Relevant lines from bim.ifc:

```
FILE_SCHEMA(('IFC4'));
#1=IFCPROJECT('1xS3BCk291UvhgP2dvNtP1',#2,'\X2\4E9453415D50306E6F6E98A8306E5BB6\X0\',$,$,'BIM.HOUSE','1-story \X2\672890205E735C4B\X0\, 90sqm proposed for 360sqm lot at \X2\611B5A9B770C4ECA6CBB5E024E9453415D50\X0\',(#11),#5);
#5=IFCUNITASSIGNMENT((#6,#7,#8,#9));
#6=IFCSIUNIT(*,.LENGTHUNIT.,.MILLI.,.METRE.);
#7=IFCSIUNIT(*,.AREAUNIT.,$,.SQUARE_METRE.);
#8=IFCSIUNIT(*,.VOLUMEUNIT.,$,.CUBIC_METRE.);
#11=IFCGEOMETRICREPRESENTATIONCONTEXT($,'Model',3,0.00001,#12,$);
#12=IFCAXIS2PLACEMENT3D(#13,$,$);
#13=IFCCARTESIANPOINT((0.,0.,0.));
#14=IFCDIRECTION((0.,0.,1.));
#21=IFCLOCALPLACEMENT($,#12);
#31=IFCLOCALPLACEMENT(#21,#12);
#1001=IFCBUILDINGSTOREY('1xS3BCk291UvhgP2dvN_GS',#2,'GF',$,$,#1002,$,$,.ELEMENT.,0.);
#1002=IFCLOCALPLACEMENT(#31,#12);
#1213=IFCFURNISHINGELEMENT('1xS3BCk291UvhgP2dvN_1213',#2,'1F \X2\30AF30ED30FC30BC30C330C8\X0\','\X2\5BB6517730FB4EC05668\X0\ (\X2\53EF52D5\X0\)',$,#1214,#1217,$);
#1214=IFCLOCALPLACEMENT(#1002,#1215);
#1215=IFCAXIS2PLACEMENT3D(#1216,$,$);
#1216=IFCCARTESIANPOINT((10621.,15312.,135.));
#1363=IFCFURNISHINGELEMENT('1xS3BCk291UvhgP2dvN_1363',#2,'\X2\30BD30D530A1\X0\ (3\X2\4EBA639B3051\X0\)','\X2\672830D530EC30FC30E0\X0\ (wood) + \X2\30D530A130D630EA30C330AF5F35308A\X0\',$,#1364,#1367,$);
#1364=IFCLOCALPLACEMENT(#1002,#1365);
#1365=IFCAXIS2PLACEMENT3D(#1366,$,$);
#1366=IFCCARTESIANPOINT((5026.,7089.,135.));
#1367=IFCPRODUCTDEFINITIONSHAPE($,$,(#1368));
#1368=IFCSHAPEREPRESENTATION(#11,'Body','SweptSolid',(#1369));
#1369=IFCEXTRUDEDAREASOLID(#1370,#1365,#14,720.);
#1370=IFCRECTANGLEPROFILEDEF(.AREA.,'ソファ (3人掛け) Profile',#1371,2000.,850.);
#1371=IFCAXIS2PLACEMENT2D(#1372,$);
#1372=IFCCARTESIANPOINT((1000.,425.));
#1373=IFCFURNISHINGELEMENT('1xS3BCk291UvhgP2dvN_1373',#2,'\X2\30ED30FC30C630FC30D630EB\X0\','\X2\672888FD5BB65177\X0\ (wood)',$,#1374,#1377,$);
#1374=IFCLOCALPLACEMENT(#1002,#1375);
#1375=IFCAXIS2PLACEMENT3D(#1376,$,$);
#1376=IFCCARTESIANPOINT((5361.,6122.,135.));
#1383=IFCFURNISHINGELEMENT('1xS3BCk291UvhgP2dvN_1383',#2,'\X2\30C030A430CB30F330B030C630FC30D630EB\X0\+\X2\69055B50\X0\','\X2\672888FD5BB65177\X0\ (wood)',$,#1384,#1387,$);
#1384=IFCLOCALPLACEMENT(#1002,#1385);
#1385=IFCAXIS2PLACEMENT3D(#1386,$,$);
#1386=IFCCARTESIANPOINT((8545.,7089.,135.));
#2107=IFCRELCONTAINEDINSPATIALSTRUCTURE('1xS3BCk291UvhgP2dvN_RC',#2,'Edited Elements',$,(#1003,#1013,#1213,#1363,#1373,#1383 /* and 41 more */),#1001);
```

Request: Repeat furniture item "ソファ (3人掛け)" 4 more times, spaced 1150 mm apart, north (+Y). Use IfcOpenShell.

```python
import numpy as np
import ifcopenshell
import ifcopenshell.api.geometry
import ifcopenshell.api.root
import ifcopenshell.util.element
import ifcopenshell.util.placement

model = ifcopenshell.open("bim.ifc")


def reuse_history(source, copy):
    """copy_class also copies each property set's owner history, people and application; keep the originals."""
    for rel in copy.IsDefinedBy:
        if rel.is_a("IfcRelDefinesByProperties") and (history := rel.RelatingPropertyDefinition.OwnerHistory):
            rel.RelatingPropertyDefinition.OwnerHistory = source.OwnerHistory
            ifcopenshell.util.element.remove_deep2(model, history)


source = model.by_id(1363)
base = ifcopenshell.util.placement.get_local_placement(source.ObjectPlacement)
step = np.array([0.0, 1.0, 0.0]) * 1150.0

for i in range(1, 5):
    copy = ifcopenshell.api.root.copy_class(model, product=source)
    copy.Representation = ifcopenshell.util.element.copy_deep(
        model, source.Representation, exclude=["IfcGeometricRepresentationContext", "IfcRepresentationMap"]
    )
    reuse_history(source, copy)
    matrix = base.copy()
    matrix[:3, 3] += i * step
    print("added at", matrix[:3, 3].round(3) + 0.0)
    ifcopenshell.api.geometry.edit_object_placement(model, product=copy, matrix=matrix, is_si=False)

model.write("bim_v2.ifc")
```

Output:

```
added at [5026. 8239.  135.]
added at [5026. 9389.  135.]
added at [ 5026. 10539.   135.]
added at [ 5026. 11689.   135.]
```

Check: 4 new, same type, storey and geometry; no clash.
